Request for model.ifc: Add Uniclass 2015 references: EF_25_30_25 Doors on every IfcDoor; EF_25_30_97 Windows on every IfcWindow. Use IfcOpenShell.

First a look at what the model holds.

```python
import ifcopenshell

model = ifcopenshell.open("model.ifc")
print(model.schema)
print("classifications:", [c.Name for c in model.by_type("IfcClassification")])
for ifc_class in ("IfcDoor", "IfcRoof", "IfcStair", "IfcWall", "IfcWindow"):
    print(ifc_class, len(model.by_type(ifc_class)))
```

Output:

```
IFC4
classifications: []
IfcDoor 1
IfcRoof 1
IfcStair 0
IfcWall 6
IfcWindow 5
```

```python
import ifcopenshell
import ifcopenshell.api.classification

model = ifcopenshell.open("model.ifc")

system = ifcopenshell.api.classification.add_classification(model, classification="Uniclass 2015")

codes = {
    "IfcDoor": ("EF_25_30_25", "Doors"),
    "IfcWindow": ("EF_25_30_97", "Windows"),
}
for ifc_class, (code, name) in codes.items():
    products = model.by_type(ifc_class)
    ifcopenshell.api.classification.add_reference(
        model, products=products, classification=system, identification=code, name=name
    )
    print(code, len(products))

model.write("model_v2.ifc")
```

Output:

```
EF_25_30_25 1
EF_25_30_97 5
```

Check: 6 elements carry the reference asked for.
